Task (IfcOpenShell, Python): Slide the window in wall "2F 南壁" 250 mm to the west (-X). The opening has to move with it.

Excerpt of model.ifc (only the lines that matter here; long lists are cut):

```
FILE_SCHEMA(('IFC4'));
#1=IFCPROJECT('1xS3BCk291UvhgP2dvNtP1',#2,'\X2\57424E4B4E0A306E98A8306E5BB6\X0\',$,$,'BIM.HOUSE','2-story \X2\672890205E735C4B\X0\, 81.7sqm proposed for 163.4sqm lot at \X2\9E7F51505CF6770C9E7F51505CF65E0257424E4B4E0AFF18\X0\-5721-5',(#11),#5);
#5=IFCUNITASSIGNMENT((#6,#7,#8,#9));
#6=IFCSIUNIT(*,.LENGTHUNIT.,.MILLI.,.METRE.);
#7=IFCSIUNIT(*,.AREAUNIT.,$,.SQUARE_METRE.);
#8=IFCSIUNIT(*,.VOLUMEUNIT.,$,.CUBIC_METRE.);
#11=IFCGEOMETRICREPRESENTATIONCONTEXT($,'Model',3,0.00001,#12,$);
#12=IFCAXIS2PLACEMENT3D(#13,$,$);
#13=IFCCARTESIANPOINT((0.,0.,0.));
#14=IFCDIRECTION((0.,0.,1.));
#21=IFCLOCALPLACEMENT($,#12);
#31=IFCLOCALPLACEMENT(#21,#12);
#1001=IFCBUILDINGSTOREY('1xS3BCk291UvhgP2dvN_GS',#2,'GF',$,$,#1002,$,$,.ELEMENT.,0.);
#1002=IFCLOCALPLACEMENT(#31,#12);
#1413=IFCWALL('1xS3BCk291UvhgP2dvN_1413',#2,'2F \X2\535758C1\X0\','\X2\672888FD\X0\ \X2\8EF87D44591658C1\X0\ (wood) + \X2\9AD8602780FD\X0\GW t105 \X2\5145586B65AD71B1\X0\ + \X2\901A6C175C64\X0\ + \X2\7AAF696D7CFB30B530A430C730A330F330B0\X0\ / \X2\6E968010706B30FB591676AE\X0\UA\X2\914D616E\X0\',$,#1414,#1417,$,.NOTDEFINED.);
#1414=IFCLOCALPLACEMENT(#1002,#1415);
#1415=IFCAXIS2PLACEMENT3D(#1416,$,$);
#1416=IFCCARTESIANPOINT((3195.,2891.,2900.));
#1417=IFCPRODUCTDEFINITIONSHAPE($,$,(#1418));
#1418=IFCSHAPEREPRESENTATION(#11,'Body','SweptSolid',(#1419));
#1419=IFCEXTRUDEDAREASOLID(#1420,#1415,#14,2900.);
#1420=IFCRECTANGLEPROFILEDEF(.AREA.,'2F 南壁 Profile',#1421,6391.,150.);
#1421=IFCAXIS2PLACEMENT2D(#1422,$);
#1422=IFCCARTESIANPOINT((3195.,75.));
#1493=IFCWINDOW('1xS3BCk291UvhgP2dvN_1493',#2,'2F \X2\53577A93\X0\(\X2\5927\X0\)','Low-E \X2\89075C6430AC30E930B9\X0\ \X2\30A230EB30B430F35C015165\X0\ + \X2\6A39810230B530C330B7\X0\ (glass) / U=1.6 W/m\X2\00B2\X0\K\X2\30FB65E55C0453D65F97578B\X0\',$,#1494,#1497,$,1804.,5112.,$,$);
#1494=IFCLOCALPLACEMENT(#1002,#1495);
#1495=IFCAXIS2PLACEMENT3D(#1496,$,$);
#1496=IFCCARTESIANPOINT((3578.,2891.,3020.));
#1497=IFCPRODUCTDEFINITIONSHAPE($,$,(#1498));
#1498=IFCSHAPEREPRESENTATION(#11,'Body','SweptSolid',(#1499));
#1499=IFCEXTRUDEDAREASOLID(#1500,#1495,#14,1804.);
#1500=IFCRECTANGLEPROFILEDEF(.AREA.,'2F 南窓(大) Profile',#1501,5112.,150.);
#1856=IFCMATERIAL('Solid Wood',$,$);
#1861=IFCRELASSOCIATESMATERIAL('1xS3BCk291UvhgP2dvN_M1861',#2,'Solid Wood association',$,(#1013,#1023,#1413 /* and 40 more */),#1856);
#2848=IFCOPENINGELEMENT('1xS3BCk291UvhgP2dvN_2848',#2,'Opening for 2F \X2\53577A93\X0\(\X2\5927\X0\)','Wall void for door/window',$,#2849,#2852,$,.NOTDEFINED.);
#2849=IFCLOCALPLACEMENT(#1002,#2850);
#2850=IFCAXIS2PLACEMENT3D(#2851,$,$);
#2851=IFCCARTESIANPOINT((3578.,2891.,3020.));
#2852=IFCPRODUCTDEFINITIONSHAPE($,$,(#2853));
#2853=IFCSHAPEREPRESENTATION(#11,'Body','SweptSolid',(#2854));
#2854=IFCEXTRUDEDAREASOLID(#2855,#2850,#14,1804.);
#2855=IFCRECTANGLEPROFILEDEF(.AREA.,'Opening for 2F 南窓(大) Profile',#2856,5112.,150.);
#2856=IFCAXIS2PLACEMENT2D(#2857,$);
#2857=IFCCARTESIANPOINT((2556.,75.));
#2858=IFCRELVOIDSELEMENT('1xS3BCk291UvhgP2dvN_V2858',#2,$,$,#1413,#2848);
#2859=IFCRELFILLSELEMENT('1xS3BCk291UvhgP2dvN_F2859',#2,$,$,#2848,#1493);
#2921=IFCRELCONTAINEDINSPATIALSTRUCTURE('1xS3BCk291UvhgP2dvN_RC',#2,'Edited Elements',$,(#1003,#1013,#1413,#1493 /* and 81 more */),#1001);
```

```python
import ifcopenshell
import ifcopenshell.api.geometry
import ifcopenshell.util.placement

model = ifcopenshell.open("model.ifc")

window = model.by_id(1493)
opening = window.FillsVoids[0].RelatingOpeningElement
wall = opening.VoidsElements[0].RelatingBuildingElement

wall_matrix = ifcopenshell.util.placement.get_local_placement(wall.ObjectPlacement)
shift = wall_matrix[:3, 0] * -250.0
before = ifcopenshell.util.placement.get_local_placement(window.ObjectPlacement)[:3, 3].copy()

# The window is not placed relative to its opening, so move both.
for product in (opening, window):
    matrix = ifcopenshell.util.placement.get_local_placement(product.ObjectPlacement)
    matrix[:3, 3] += shift
    ifcopenshell.api.geometry.edit_object_placement(model, product=product, matrix=matrix, is_si=False)

after = ifcopenshell.util.placement.get_local_placement(window.ObjectPlacement)[:3, 3]
print("window moved by", (after - before).round(3) + 0.0)

model.write("model_updated.ifc")
```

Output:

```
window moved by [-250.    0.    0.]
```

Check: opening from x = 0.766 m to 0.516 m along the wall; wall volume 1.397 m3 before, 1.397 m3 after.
